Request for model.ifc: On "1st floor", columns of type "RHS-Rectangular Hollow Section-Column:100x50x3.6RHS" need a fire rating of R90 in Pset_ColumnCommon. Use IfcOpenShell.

First a look at what the model holds.

```python
import ifcopenshell
import ifcopenshell.util.element

model = ifcopenshell.open("model.ifc")
print(model.schema)
storey = next(s for s in model.by_type("IfcBuildingStorey") if s.Name == "1st floor")
columns = [e for e in ifcopenshell.util.element.get_decomposition(storey) if e.is_a("IfcColumn")]
seen = {}
for e in columns:
    element_type = ifcopenshell.util.element.get_type(e)
    key = (element_type.Name if element_type != e and element_type else None, ifcopenshell.util.element.get_pset(e, "Pset_ColumnCommon", "FireRating"))
    seen[key] = seen.get(key, 0) + 1
for (name, value), count in sorted(seen.items(), key=str):
    print(count, "x", name, "|", value)
```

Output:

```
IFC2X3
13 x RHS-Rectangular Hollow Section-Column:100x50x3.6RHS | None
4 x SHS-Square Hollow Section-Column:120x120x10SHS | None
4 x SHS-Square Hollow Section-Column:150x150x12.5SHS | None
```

```python
import ifcopenshell
import ifcopenshell.api.pset
import ifcopenshell.util.element

model = ifcopenshell.open("model.ifc")

storey = next(s for s in model.by_type("IfcBuildingStorey") if s.Name == "1st floor")
columns = [e for e in ifcopenshell.util.element.get_decomposition(storey) if e.is_a("IfcColumn")]

count = 0
for e in columns:
    element_type = ifcopenshell.util.element.get_type(e)
    if element_type in (None, e) or element_type.Name != "RHS-Rectangular Hollow Section-Column:100x50x3.6RHS":
        continue
    # add_pset returns the element's existing set when there is one.
    pset = ifcopenshell.api.pset.add_pset(model, product=e, name="Pset_ColumnCommon")
    ifcopenshell.api.pset.edit_pset(model, pset=pset, properties={"FireRating": "R90"})
    count += 1

print(count, "columns updated")

model.write("model_edited.ifc")
```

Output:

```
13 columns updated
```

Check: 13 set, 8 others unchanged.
